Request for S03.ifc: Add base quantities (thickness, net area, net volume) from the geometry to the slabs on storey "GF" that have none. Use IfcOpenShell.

First a look at what the model holds.

```python
import ifcopenshell
import ifcopenshell.util.element
import ifcopenshell.util.unit

model = ifcopenshell.open("S03.ifc")
print(model.schema)
for unit_type in ("LENGTHUNIT", "AREAUNIT", "VOLUMEUNIT"):
    print(unit_type, ifcopenshell.util.unit.calculate_unit_scale(model, unit_type))
storey = next(s for s in model.by_type("IfcBuildingStorey") if s.Name == "GF")
slabs = [e for e in ifcopenshell.util.element.get_decomposition(storey) if e.is_a("IfcSlab")]
for e in sorted(slabs, key=lambda e: e.id()):
    print(e.id(), e.is_a(), e.Name, list(ifcopenshell.util.element.get_psets(e, qtos_only=True)), sep=" | ")
```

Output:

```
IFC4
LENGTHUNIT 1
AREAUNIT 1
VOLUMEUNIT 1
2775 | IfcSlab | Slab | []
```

```python
import ifcopenshell
import ifcopenshell.api.pset
import ifcopenshell.geom
import ifcopenshell.util.element
import ifcopenshell.util.shape
import ifcopenshell.util.unit

model = ifcopenshell.open("S03.ifc")
unit_scale = ifcopenshell.util.unit.calculate_unit_scale(model)
area_scale = ifcopenshell.util.unit.calculate_unit_scale(model, "AREAUNIT")
volume_scale = ifcopenshell.util.unit.calculate_unit_scale(model, "VOLUMEUNIT")
settings = ifcopenshell.geom.settings()

storey = next(s for s in model.by_type("IfcBuildingStorey") if s.Name == "GF")
slabs = [e for e in ifcopenshell.util.element.get_decomposition(storey) if e.is_a("IfcSlab")]

for e in sorted(slabs, key=lambda e: e.id()):
    if ifcopenshell.util.element.get_psets(e, qtos_only=True, should_inherit=False):
        continue
    # Geometry comes back in metres, in the element's own axes.
    shape = ifcopenshell.geom.create_shape(settings, e)
    values = {
        "Width": ifcopenshell.util.shape.get_z(shape.geometry) / unit_scale,
        "NetArea": ifcopenshell.util.shape.get_footprint_area(shape.geometry) / area_scale,
        "NetVolume": ifcopenshell.util.shape.get_volume(shape.geometry) / volume_scale,
    }
    qto = ifcopenshell.api.pset.add_qto(model, product=e, name="Qto_SlabBaseQuantities")
    ifcopenshell.api.pset.edit_qto(model, qto=qto, properties=values)
    print(e.id(), {k: round(v, 3) for k, v in values.items()})

model.write("S03_rev.ifc")
```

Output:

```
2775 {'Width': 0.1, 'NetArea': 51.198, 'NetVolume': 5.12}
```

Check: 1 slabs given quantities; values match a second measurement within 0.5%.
